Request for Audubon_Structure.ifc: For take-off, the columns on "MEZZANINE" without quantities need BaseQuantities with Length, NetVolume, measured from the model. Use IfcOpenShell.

First a look at what the model holds.

```python
import ifcopenshell
import ifcopenshell.util.element
import ifcopenshell.util.unit

model = ifcopenshell.open("Audubon_Structure.ifc")
print(model.schema)
for unit_type in ("LENGTHUNIT", "AREAUNIT", "VOLUMEUNIT"):
    print(unit_type, ifcopenshell.util.unit.calculate_unit_scale(model, unit_type))
storey = next(s for s in model.by_type("IfcBuildingStorey") if s.Name == "MEZZANINE")
columns = [e for e in ifcopenshell.util.element.get_decomposition(storey) if e.is_a("IfcColumn")]
for e in sorted(columns, key=lambda e: e.id()):
    print(e.id(), e.is_a(), e.Name, list(ifcopenshell.util.element.get_psets(e, qtos_only=True)), sep=" | ")
```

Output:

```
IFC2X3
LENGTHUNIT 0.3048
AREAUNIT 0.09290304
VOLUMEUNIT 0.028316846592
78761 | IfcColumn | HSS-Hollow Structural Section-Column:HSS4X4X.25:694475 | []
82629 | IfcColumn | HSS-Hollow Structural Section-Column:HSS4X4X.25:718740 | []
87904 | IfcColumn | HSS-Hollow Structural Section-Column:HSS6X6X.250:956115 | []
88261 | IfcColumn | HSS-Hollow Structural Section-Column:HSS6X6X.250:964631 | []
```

```python
import ifcopenshell
import ifcopenshell.api.pset
import ifcopenshell.geom
import ifcopenshell.util.element
import ifcopenshell.util.shape
import ifcopenshell.util.unit

model = ifcopenshell.open("Audubon_Structure.ifc")
unit_scale = ifcopenshell.util.unit.calculate_unit_scale(model)
volume_scale = ifcopenshell.util.unit.calculate_unit_scale(model, "VOLUMEUNIT")
settings = ifcopenshell.geom.settings()

storey = next(s for s in model.by_type("IfcBuildingStorey") if s.Name == "MEZZANINE")
columns = [e for e in ifcopenshell.util.element.get_decomposition(storey) if e.is_a("IfcColumn")]

for e in sorted(columns, key=lambda e: e.id()):
    if ifcopenshell.util.element.get_psets(e, qtos_only=True, should_inherit=False):
        continue
    # Geometry comes back in metres, in the element's own axes.
    shape = ifcopenshell.geom.create_shape(settings, e)
    values = {
        "Length": ifcopenshell.util.shape.get_z(shape.geometry) / unit_scale,
        "NetVolume": ifcopenshell.util.shape.get_volume(shape.geometry) / volume_scale,
    }
    qto = ifcopenshell.api.pset.add_qto(model, product=e, name="BaseQuantities")
    ifcopenshell.api.pset.edit_qto(model, qto=qto, properties=values)
    print(e.id(), {k: round(v, 3) for k, v in values.items()})

model.write("Audubon_Structure_v2.ifc")
```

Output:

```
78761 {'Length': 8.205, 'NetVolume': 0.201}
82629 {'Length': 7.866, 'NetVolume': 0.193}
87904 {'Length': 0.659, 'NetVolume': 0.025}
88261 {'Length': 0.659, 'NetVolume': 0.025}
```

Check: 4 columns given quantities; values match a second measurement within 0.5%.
